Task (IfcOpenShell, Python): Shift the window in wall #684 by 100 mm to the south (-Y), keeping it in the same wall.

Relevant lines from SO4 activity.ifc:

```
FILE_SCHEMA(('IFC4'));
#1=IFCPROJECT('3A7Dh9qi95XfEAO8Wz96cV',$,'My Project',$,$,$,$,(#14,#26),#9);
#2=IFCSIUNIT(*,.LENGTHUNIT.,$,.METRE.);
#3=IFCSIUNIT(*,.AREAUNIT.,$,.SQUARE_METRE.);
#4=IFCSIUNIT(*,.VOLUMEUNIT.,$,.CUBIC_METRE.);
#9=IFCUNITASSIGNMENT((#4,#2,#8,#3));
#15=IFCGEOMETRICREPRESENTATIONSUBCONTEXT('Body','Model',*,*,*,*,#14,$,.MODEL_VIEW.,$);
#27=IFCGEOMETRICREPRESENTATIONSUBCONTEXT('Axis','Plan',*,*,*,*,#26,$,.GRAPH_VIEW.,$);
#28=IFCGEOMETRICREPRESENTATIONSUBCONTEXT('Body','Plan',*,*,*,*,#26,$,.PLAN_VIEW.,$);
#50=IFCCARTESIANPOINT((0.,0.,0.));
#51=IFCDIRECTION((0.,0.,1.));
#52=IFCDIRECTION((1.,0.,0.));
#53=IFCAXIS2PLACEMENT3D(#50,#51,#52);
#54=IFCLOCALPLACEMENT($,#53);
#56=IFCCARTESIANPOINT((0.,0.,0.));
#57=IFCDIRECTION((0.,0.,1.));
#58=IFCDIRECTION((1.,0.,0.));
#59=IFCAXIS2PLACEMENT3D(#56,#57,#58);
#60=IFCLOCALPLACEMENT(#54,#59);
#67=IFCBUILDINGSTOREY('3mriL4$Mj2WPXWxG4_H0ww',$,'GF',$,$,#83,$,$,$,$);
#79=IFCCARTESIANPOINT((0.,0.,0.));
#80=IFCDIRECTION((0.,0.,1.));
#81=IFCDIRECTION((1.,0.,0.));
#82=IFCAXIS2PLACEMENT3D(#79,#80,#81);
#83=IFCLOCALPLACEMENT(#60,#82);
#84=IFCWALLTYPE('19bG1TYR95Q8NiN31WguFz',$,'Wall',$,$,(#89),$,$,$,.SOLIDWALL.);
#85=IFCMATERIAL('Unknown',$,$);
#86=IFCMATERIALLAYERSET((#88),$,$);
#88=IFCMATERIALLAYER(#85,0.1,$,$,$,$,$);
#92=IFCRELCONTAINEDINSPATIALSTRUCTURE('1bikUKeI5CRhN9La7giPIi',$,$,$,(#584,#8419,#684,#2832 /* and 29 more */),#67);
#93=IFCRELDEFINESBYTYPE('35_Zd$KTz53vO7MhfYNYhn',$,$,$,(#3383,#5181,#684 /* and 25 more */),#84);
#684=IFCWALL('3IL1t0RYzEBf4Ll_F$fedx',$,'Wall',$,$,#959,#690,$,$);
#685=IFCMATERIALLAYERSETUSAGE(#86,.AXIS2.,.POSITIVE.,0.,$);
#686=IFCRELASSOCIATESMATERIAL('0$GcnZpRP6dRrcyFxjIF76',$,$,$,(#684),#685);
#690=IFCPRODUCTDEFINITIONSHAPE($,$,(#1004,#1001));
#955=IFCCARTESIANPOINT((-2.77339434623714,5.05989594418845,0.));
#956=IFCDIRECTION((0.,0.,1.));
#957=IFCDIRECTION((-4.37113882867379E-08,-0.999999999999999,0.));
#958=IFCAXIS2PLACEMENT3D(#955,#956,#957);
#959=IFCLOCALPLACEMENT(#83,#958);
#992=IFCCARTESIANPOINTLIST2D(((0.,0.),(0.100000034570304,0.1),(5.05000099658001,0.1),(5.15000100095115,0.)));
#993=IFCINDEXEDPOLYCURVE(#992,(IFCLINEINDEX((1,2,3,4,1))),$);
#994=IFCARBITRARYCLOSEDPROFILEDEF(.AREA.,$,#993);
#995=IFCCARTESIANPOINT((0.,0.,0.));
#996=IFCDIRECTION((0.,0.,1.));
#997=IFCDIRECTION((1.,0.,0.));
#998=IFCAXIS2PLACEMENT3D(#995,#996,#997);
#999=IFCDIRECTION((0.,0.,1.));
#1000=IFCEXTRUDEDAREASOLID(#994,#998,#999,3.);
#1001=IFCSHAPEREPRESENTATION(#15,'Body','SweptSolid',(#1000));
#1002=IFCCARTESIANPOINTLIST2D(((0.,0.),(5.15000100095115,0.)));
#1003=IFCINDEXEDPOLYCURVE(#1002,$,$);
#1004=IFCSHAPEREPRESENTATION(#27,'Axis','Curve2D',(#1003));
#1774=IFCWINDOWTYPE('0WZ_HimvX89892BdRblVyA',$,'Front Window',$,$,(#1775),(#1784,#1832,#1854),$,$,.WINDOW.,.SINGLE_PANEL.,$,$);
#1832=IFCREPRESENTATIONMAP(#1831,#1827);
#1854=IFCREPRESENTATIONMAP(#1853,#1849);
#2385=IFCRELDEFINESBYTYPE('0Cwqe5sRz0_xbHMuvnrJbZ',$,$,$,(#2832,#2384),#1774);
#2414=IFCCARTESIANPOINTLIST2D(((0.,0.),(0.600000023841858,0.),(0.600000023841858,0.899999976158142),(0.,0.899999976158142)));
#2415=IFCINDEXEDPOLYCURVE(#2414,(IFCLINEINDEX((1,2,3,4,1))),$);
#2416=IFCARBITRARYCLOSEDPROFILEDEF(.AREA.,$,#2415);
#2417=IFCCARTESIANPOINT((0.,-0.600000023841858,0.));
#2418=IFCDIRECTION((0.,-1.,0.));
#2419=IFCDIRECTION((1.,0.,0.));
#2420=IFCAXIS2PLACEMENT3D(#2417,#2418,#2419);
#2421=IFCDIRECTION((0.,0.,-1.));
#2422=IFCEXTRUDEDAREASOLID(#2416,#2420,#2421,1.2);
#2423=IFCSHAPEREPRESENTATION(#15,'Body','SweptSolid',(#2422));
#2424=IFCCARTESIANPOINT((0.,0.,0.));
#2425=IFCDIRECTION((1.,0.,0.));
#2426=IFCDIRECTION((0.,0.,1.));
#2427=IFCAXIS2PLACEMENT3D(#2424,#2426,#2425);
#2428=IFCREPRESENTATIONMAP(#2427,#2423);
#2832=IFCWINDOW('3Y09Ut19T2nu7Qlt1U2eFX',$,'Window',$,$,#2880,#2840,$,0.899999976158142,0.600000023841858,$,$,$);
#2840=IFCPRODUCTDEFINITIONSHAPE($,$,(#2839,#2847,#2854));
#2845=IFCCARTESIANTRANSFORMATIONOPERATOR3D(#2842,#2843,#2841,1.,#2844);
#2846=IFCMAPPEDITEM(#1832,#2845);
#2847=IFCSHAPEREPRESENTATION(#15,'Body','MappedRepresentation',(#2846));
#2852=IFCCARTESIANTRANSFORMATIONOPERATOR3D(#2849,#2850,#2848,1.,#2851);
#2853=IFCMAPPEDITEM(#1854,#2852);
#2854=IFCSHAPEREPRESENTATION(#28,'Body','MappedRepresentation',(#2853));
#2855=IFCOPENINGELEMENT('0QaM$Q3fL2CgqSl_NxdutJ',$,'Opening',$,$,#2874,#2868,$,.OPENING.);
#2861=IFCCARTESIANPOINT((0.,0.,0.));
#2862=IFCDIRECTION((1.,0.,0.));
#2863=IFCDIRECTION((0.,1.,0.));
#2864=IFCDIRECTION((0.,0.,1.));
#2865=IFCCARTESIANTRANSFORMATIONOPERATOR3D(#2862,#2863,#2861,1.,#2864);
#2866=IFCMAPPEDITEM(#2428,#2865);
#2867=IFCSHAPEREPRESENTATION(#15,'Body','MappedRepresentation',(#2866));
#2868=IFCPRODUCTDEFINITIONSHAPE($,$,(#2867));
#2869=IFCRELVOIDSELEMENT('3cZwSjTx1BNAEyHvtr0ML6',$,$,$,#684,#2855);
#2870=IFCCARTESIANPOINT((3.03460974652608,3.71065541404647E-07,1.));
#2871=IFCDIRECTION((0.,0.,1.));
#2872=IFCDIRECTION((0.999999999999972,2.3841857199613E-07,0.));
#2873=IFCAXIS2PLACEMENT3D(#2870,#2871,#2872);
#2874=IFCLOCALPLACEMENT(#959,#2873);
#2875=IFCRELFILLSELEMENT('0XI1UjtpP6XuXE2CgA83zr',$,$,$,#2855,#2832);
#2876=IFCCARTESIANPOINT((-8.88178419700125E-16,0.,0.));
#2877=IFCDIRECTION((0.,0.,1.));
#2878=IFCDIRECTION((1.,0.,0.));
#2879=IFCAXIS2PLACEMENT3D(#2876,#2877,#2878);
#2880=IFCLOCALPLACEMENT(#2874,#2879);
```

```python
import ifcopenshell
import ifcopenshell.api.geometry
import ifcopenshell.util.placement
import ifcopenshell.util.unit

model = ifcopenshell.open("SO4 activity.ifc")
unit_scale = ifcopenshell.util.unit.calculate_unit_scale(model)

window = model.by_guid("3Y09Ut19T2nu7Qlt1U2eFX")
opening = window.FillsVoids[0].RelatingOpeningElement
wall = opening.VoidsElements[0].RelatingBuildingElement

wall_matrix = ifcopenshell.util.placement.get_local_placement(wall.ObjectPlacement)
shift = wall_matrix[:3, 0] * 0.1 / unit_scale
before = ifcopenshell.util.placement.get_local_placement(window.ObjectPlacement)[:3, 3].copy()

# The window is placed relative to its opening, so it follows when the opening moves.
matrix = ifcopenshell.util.placement.get_local_placement(opening.ObjectPlacement)
matrix[:3, 3] += shift
ifcopenshell.api.geometry.edit_object_placement(
    model, product=opening, matrix=matrix, is_si=False, should_transform_children=True
)

after = ifcopenshell.util.placement.get_local_placement(window.ObjectPlacement)[:3, 3]
print("window moved by", (after - before).round(3) + 0.0)

model.write("SO4 activity_edited.ifc")
```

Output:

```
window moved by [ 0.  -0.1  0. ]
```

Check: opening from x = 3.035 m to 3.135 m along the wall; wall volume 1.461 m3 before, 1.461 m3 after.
